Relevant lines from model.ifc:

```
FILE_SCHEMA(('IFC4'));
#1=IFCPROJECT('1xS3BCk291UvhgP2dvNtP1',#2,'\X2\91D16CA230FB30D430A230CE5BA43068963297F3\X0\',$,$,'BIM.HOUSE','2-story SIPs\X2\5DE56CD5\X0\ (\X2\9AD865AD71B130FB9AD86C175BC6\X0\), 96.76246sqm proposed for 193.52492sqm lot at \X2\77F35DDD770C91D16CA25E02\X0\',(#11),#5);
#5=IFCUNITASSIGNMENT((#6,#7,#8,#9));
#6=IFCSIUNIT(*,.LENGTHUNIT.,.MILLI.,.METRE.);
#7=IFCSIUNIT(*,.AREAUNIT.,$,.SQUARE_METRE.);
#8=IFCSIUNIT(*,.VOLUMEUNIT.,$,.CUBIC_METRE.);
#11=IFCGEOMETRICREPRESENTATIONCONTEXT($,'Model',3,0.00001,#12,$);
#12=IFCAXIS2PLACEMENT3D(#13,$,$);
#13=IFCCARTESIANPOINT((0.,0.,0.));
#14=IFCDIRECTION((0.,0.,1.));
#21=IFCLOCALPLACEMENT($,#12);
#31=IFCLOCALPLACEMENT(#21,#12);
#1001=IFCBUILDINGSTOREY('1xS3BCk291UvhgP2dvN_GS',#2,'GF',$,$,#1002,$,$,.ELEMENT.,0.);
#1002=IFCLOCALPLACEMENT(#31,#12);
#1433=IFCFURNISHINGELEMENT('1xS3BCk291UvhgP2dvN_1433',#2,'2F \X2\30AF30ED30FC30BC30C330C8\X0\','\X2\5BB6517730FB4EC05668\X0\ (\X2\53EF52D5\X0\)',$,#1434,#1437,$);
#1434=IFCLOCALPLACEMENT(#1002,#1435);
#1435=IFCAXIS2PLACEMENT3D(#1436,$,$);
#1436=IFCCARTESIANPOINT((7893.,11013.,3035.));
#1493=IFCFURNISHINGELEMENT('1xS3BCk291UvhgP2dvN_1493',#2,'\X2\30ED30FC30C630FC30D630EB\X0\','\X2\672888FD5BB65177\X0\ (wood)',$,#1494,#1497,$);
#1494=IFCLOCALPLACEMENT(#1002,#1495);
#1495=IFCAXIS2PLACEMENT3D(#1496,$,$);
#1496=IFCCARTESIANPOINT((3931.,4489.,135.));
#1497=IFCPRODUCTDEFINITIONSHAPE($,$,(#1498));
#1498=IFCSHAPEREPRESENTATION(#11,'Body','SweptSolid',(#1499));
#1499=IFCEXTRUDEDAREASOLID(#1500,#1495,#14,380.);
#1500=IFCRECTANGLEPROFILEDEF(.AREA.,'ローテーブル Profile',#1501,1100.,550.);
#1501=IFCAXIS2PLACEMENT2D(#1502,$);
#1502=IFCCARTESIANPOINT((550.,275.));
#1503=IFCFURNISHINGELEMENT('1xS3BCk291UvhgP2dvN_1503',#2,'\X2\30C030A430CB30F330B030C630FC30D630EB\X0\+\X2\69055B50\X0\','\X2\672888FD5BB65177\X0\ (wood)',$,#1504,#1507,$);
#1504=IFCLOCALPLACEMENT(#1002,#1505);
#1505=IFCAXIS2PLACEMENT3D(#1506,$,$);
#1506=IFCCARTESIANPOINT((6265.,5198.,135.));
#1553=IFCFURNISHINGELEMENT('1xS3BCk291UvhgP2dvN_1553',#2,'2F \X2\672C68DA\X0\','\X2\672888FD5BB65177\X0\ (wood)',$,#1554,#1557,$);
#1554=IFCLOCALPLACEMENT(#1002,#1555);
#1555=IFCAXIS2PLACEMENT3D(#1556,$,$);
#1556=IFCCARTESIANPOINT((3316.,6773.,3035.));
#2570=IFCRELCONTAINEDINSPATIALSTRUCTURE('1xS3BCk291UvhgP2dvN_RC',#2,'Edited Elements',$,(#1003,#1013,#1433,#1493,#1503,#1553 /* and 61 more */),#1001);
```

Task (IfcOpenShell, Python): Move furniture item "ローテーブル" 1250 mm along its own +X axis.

```python
import ifcopenshell
import ifcopenshell.api.geometry
import ifcopenshell.util.placement

model = ifcopenshell.open("model.ifc")

item = model.by_guid("1xS3BCk291UvhgP2dvN_1493")
matrix = ifcopenshell.util.placement.get_local_placement(item.ObjectPlacement)
matrix[:3, 3] += matrix[:3, 0] * 1250.0
ifcopenshell.api.geometry.edit_object_placement(model, product=item, matrix=matrix, is_si=False)

print(ifcopenshell.util.placement.get_local_placement(item.ObjectPlacement).round(3) + 0.0)

model.write("model_updated.ifc")
```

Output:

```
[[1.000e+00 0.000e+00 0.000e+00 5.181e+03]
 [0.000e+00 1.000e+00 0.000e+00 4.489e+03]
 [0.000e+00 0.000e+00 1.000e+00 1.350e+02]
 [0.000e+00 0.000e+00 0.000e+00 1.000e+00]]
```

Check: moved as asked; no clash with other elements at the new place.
